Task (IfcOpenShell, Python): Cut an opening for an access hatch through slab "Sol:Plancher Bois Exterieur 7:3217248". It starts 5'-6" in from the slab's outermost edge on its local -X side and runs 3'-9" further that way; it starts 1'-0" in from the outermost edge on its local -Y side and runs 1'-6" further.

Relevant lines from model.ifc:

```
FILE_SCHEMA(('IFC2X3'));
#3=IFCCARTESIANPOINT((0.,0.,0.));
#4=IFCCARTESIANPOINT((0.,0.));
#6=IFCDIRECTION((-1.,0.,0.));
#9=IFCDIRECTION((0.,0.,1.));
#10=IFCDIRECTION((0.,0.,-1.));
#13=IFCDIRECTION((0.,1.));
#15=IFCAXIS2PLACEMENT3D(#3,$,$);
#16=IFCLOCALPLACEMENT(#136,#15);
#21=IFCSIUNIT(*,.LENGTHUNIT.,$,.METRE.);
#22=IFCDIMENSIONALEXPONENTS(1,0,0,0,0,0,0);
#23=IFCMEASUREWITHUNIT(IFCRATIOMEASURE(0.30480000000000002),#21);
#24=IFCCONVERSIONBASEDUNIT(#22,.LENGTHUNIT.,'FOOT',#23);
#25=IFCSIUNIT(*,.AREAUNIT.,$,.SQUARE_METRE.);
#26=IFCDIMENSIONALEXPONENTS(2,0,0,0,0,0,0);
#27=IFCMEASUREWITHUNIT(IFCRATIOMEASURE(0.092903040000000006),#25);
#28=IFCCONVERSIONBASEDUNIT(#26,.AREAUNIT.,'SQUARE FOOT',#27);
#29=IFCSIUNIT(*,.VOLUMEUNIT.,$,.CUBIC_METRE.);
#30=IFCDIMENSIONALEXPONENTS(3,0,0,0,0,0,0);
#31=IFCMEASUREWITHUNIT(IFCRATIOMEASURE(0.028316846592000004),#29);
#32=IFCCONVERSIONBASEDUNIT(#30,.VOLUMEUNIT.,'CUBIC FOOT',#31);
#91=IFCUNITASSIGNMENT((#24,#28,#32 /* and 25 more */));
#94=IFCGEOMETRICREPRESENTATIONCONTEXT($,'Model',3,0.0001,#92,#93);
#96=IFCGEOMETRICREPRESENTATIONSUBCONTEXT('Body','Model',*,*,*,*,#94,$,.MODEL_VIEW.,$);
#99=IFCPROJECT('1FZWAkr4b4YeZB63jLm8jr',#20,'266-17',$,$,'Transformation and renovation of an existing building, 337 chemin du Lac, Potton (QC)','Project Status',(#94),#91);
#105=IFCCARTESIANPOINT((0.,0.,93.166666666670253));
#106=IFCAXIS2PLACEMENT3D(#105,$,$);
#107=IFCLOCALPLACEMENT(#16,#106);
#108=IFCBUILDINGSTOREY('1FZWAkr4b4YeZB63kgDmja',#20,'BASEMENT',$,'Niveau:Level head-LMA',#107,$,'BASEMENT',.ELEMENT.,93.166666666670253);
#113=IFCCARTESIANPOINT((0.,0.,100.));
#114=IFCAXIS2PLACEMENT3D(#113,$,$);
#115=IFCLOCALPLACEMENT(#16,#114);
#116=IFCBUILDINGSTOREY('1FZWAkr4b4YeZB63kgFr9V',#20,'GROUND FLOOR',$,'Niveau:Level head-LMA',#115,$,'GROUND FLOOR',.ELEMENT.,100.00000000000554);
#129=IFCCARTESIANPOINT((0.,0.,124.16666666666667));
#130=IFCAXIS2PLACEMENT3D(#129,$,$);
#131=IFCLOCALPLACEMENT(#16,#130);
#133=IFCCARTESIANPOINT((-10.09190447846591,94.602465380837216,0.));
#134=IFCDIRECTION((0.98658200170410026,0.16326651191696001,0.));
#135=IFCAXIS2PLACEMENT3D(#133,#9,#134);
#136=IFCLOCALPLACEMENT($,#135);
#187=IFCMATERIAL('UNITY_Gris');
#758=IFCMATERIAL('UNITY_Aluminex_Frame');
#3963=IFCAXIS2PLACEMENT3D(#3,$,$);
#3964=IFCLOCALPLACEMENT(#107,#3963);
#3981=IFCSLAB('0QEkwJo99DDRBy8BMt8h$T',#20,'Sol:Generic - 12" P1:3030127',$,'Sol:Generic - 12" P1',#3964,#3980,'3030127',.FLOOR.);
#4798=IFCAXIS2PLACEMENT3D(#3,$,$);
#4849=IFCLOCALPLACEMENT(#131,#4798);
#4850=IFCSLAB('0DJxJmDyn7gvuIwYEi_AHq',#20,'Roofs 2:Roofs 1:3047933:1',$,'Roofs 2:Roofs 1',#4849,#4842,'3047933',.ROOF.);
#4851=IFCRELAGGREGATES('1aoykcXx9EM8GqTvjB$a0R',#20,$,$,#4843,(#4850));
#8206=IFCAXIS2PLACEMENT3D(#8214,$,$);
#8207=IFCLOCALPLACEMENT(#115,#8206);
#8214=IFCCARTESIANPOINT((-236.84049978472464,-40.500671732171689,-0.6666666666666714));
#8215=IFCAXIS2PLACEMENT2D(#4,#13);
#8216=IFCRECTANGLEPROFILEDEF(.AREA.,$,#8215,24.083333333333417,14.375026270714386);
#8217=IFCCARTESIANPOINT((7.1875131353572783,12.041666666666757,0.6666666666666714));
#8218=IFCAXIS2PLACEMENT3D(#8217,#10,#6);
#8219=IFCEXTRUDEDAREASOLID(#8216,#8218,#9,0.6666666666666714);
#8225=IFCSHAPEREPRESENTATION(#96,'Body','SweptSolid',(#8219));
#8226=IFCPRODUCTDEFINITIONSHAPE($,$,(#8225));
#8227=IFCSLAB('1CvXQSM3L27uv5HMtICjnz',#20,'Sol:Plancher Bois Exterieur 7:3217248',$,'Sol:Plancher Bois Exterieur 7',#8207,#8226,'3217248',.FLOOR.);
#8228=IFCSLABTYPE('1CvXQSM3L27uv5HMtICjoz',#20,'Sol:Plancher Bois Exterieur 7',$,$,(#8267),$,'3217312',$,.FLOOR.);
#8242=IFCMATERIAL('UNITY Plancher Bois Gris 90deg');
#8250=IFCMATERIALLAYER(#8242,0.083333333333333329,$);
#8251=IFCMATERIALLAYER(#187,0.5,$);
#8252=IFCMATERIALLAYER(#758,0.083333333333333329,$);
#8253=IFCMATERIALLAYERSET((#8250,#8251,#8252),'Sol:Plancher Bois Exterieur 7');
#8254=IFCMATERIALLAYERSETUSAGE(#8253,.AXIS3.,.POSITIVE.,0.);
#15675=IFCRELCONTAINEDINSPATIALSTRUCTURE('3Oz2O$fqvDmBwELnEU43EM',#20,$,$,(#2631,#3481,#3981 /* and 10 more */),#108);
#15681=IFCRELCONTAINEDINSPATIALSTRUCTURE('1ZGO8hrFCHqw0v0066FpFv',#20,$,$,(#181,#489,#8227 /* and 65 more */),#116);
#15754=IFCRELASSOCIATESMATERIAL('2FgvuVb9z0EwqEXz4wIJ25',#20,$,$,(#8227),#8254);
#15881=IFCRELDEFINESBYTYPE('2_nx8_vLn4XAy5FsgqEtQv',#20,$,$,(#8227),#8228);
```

```python
import numpy as np
import ifcopenshell
import ifcopenshell.api.feature
import ifcopenshell.api.geometry
import ifcopenshell.api.root
import ifcopenshell.geom
import ifcopenshell.util.placement
import ifcopenshell.util.representation
import ifcopenshell.util.shape
import ifcopenshell.util.unit

model = ifcopenshell.open("model.ifc")
unit_scale = ifcopenshell.util.unit.calculate_unit_scale(model)
settings = ifcopenshell.geom.settings()


def volume(element):
    """Net volume in cubic metres, openings subtracted."""
    shape = ifcopenshell.geom.create_shape(settings, element)
    return ifcopenshell.util.shape.get_volume(shape.geometry)


slab = model.by_id(8227)
before = volume(slab)

# Extent in the slab's own axes, in metres. The edges named are its -X and -Y sides.
slab_shape = ifcopenshell.geom.create_shape(settings, slab)
vertices = ifcopenshell.util.shape.get_vertices(slab_shape.geometry)
x_min, y_min, bottom = vertices.min(axis=0)
top = vertices[:, 2].max()

opening = ifcopenshell.api.root.create_entity(model, ifc_class="IfcOpeningElement", name="Access hatch opening")
context = ifcopenshell.util.representation.get_context(model, "Model", "Body", "MODEL_VIEW")
width, depth = 1.143, 0.4572
outline = [(0.0, 0.0), (width, 0.0), (width, depth), (0.0, depth), (0.0, 0.0)]
# Overshoot both faces by 50 mm so the cut is clean.
shape = ifcopenshell.api.geometry.add_slab_representation(
    model, context=context, depth=top - bottom + 0.1, polyline=outline
)
ifcopenshell.api.geometry.assign_representation(model, product=opening, representation=shape)

matrix = ifcopenshell.util.placement.get_local_placement(slab.ObjectPlacement)
matrix[:, 3] = matrix @ np.append(np.array([x_min + 1.6764, y_min + 0.3048, bottom - 0.05]) / unit_scale, 1.0)
ifcopenshell.api.geometry.edit_object_placement(model, product=opening, matrix=matrix, is_si=False)
ifcopenshell.api.feature.add_feature(model, feature=opening, element=slab)

after = volume(slab)

print(f"slab volume {before:.3f} -> {after:.3f} m3")

model.write("model_v2.ifc")
```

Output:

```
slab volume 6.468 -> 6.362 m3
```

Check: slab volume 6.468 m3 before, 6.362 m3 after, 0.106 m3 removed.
